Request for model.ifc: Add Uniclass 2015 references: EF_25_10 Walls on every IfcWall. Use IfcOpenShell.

First a look at what the model holds.

```python
import ifcopenshell

model = ifcopenshell.open("model.ifc")
print(model.schema)
print("classifications:", [c.Name for c in model.by_type("IfcClassification")])
for ifc_class in ("IfcDoor", "IfcRoof", "IfcStair", "IfcWall", "IfcWindow"):
    print(ifc_class, len(model.by_type(ifc_class)))
```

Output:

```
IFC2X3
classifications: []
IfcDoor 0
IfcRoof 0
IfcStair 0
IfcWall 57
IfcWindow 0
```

```python
import ifcopenshell
import ifcopenshell.api.classification

model = ifcopenshell.open("model.ifc")

# IFC2X3 requires Source and Edition and has no link from the project to the system.
system = model.create_entity("IfcClassification", Source="NBS", Edition="2015", Name="Uniclass 2015")

codes = {
    "IfcWall": ("EF_25_10", "Walls"),
}
for ifc_class, (code, name) in codes.items():
    products = model.by_type(ifc_class)
    ifcopenshell.api.classification.add_reference(
        model, products=products, classification=system, identification=code, name=name
    )
    print(code, len(products))

model.write("model_edited.ifc")
```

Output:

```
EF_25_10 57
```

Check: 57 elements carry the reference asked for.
